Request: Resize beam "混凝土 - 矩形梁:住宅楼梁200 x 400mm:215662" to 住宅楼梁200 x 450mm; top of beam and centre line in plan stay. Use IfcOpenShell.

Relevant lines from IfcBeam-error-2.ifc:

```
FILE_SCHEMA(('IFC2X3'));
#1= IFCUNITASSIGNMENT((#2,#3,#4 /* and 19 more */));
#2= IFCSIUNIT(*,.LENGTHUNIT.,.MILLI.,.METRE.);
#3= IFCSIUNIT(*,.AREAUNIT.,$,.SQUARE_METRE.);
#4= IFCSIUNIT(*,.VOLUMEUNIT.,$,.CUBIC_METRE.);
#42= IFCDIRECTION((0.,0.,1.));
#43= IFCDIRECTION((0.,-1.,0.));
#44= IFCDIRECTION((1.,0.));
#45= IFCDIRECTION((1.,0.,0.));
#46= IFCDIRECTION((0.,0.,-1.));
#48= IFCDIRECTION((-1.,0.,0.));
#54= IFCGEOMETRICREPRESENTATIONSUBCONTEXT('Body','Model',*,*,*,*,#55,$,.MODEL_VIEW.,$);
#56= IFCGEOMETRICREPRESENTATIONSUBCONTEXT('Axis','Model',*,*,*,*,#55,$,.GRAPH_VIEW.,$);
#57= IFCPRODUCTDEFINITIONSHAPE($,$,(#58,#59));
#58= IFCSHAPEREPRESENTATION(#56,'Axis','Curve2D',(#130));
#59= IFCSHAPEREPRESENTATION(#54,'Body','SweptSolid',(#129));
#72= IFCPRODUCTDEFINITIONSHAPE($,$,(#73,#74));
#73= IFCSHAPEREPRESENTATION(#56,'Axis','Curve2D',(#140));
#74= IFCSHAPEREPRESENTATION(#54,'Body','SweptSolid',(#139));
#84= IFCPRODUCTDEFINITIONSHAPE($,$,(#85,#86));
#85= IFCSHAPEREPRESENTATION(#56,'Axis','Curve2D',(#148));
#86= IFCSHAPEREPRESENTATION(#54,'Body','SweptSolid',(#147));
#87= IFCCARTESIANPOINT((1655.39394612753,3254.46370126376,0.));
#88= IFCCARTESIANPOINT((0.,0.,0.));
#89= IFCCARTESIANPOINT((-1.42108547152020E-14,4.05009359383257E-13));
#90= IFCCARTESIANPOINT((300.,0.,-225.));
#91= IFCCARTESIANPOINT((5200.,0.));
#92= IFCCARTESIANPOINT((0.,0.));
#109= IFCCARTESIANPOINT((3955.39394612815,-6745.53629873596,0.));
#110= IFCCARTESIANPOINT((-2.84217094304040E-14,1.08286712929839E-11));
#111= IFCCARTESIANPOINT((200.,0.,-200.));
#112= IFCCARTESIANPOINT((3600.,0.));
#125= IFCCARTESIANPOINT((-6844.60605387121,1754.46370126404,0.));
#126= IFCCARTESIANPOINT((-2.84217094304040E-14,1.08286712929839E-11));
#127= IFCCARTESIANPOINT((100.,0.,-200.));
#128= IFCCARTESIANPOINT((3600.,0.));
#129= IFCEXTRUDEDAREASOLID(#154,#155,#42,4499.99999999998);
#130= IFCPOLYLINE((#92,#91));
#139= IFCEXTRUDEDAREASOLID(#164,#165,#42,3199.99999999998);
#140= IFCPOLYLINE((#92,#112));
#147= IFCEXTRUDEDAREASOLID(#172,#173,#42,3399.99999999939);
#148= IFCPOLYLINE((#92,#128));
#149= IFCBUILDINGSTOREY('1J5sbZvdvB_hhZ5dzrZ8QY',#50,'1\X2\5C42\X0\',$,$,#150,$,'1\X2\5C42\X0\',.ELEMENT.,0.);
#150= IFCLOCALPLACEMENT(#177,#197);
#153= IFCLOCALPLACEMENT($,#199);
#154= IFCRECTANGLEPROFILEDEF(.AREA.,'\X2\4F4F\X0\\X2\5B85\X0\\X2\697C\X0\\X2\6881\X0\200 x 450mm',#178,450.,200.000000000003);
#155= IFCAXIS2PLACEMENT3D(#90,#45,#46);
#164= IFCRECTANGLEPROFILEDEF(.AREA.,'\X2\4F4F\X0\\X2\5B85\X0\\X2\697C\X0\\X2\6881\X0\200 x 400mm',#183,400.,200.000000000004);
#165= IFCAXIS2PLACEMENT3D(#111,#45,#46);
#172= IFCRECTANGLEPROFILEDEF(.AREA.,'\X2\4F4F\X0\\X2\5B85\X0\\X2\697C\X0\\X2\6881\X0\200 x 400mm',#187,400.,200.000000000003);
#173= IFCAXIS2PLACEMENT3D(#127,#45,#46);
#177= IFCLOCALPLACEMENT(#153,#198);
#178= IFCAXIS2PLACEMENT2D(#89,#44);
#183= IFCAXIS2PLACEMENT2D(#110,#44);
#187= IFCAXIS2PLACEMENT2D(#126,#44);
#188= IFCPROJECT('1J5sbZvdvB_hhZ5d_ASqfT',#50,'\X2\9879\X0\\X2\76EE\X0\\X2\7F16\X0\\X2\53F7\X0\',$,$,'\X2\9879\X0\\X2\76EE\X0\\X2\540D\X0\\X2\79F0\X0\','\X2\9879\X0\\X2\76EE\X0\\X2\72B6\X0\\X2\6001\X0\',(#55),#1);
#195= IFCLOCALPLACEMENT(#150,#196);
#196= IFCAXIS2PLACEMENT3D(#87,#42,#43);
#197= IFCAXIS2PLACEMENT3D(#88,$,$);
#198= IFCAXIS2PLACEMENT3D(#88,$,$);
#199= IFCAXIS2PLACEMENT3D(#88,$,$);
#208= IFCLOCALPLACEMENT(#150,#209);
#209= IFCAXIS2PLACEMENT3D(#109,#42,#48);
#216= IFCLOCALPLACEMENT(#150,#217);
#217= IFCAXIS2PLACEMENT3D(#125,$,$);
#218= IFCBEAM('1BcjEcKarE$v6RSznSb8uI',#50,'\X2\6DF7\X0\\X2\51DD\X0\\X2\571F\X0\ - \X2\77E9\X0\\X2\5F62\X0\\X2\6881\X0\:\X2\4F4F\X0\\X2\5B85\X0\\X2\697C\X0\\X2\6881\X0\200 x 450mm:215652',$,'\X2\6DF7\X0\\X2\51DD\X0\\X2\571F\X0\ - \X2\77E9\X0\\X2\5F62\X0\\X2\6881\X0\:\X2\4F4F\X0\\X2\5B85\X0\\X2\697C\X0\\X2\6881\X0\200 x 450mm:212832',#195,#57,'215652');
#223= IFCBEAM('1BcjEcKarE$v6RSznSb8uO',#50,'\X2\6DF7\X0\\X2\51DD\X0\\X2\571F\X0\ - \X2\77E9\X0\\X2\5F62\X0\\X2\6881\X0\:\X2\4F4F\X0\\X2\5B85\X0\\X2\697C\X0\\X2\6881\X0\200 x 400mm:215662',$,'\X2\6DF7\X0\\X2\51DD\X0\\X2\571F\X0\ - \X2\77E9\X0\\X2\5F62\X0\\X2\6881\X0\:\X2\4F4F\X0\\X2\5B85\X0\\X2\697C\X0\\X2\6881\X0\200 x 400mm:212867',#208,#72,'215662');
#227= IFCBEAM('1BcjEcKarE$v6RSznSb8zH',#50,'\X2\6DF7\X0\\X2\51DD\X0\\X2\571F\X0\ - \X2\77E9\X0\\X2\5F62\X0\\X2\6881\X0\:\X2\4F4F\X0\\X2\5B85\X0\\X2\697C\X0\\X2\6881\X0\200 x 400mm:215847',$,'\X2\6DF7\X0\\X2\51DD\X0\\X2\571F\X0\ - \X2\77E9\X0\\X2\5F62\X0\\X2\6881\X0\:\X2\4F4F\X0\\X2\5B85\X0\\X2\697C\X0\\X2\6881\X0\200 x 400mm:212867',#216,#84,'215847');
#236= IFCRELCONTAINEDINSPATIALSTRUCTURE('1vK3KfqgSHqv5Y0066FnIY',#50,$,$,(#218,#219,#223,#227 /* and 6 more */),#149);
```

```python
import ifcopenshell
import ifcopenshell.util.element
import ifcopenshell.util.representation

model = ifcopenshell.open("IfcBeam-error-2.ifc")

member = model.by_id(223)
source = next(p for p in model.by_type("IfcRectangleProfileDef") if p.ProfileName == "住宅楼梁200 x 450mm")

body = ifcopenshell.util.representation.get_representation(member, "Model", "Body")
solid = body.Items[0]
old_profile = solid.SweptArea

# Copy the section's sizes but keep this member's own profile position.
profile = ifcopenshell.util.element.copy(model, source)
# Profiles are centred, so shift by half the change in depth to hold the top.
shift = (old_profile.XDim - profile.XDim) / 2
x, y = old_profile.Position.Location.Coordinates
up = (-1.0, 0.0)  # upwards, in the solid's own plane
location = model.createIfcCartesianPoint((x + up[0] * shift, y + up[1] * shift))
profile.Position = model.createIfcAxis2Placement2D(location, old_profile.Position.RefDirection)
solid.SweptArea = profile
if not model.get_total_inverses(old_profile):
    ifcopenshell.util.element.remove_deep2(model, old_profile)
member.Name = member.Name.replace("住宅楼梁200 x 400mm", "住宅楼梁200 x 450mm")
member.ObjectType = member.ObjectType.replace("住宅楼梁200 x 400mm", "住宅楼梁200 x 450mm")

print(solid.SweptArea)

model.write("IfcBeam-error-2_edited.ifc")
```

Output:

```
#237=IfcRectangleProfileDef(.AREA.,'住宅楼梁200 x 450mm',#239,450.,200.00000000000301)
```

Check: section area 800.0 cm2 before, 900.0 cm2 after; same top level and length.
